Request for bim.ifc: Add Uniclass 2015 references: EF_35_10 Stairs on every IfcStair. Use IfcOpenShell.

First a look at what the model holds.

```python
import ifcopenshell

model = ifcopenshell.open("bim.ifc")
print(model.schema)
print("classifications:", [c.Name for c in model.by_type("IfcClassification")])
for ifc_class in ("IfcDoor", "IfcRoof", "IfcStair", "IfcWall", "IfcWindow"):
    print(ifc_class, len(model.by_type(ifc_class)))
```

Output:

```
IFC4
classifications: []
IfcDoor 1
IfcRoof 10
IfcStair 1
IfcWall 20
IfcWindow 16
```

```python
import ifcopenshell
import ifcopenshell.api.classification

model = ifcopenshell.open("bim.ifc")

system = ifcopenshell.api.classification.add_classification(model, classification="Uniclass 2015")

codes = {
    "IfcStair": ("EF_35_10", "Stairs"),
}
for ifc_class, (code, name) in codes.items():
    products = model.by_type(ifc_class)
    ifcopenshell.api.classification.add_reference(
        model, products=products, classification=system, identification=code, name=name
    )
    print(code, len(products))

model.write("bim_edited.ifc")
```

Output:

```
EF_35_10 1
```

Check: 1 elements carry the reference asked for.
